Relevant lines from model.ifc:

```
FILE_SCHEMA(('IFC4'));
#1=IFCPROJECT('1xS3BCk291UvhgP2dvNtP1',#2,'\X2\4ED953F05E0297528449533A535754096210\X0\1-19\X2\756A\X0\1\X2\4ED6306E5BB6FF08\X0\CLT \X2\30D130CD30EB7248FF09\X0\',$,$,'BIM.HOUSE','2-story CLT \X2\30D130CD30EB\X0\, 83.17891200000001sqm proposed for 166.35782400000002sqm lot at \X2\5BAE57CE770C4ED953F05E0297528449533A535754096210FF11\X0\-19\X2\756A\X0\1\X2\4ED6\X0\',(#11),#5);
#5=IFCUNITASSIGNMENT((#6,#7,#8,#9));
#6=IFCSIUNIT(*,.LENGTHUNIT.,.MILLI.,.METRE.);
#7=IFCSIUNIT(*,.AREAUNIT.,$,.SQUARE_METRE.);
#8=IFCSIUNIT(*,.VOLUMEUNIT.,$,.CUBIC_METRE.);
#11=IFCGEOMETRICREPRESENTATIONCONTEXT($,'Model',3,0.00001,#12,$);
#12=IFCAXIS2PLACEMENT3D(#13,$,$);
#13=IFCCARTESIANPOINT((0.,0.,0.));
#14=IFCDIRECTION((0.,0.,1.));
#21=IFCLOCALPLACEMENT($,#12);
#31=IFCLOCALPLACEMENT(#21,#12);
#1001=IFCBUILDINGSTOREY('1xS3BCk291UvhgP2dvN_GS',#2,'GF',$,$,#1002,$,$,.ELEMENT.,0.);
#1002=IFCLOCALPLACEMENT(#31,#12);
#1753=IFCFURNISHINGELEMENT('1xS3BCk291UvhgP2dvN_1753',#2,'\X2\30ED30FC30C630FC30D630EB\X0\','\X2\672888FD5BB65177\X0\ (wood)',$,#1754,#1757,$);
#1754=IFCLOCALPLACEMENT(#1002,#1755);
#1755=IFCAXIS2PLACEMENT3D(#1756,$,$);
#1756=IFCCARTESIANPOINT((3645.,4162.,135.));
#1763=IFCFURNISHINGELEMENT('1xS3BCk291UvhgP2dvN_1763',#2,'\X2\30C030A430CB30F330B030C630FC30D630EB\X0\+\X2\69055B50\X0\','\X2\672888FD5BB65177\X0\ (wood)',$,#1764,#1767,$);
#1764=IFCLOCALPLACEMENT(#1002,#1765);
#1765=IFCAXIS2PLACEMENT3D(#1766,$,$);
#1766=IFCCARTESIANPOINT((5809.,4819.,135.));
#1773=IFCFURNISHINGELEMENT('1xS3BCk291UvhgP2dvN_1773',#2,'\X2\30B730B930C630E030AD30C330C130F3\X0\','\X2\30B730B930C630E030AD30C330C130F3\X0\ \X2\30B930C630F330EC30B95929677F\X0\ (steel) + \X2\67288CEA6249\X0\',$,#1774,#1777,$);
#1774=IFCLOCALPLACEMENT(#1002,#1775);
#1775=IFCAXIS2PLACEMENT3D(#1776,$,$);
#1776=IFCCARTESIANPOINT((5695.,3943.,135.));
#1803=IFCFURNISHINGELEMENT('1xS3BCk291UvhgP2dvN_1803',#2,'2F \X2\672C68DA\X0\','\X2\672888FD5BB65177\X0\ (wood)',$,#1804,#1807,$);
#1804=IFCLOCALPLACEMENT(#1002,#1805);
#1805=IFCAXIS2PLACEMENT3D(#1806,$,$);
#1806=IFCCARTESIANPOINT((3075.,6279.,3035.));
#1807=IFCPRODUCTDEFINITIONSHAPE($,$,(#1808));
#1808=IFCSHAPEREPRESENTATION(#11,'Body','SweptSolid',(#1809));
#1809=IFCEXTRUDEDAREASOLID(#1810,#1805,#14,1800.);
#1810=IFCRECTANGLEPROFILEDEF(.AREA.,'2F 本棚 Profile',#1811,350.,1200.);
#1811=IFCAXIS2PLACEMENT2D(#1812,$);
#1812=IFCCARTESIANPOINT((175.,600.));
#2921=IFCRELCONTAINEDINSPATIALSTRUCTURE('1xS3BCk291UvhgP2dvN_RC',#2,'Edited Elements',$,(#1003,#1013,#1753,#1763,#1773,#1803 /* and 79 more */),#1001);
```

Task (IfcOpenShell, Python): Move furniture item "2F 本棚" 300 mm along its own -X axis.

```python
import ifcopenshell
import ifcopenshell.api.geometry
import ifcopenshell.util.placement
import ifcopenshell.util.unit

model = ifcopenshell.open("model.ifc")
unit_scale = ifcopenshell.util.unit.calculate_unit_scale(model)

item = model.by_guid("1xS3BCk291UvhgP2dvN_1803")
matrix = ifcopenshell.util.placement.get_local_placement(item.ObjectPlacement)
matrix[:3, 3] -= matrix[:3, 0] * 0.3 / unit_scale
ifcopenshell.api.geometry.edit_object_placement(model, product=item, matrix=matrix, is_si=False)

print(ifcopenshell.util.placement.get_local_placement(item.ObjectPlacement).round(3) + 0.0)

model.write("model_v2.ifc")
```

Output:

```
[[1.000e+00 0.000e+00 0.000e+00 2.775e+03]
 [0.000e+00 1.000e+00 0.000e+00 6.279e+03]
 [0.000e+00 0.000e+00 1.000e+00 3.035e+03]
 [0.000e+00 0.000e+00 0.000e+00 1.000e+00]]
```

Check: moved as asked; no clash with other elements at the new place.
